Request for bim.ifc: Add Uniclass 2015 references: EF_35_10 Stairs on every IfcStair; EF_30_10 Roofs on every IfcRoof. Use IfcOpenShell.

First a look at what the model holds.

```python
import ifcopenshell

model = ifcopenshell.open("bim.ifc")
print(model.schema)
print("classifications:", [c.Name for c in model.by_type("IfcClassification")])
for ifc_class in ("IfcDoor", "IfcRoof", "IfcStair", "IfcWall", "IfcWindow"):
    print(ifc_class, len(model.by_type(ifc_class)))
```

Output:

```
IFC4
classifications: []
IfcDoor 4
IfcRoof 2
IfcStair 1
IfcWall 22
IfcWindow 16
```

```python
import ifcopenshell
import ifcopenshell.api.classification

model = ifcopenshell.open("bim.ifc")

system = ifcopenshell.api.classification.add_classification(model, classification="Uniclass 2015")

codes = {
    "IfcStair": ("EF_35_10", "Stairs"),
    "IfcRoof": ("EF_30_10", "Roofs"),
}
for ifc_class, (code, name) in codes.items():
    products = model.by_type(ifc_class)
    ifcopenshell.api.classification.add_reference(
        model, products=products, classification=system, identification=code, name=name
    )
    print(code, len(products))

model.write("bim_v2.ifc")
```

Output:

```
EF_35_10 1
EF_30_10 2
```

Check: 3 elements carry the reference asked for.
